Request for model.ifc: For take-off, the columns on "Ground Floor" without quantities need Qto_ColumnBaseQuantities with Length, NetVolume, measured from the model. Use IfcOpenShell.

First a look at what the model holds.

```python
import ifcopenshell
import ifcopenshell.util.element
import ifcopenshell.util.unit

model = ifcopenshell.open("model.ifc")
print(model.schema)
for unit_type in ("LENGTHUNIT", "AREAUNIT", "VOLUMEUNIT"):
    print(unit_type, ifcopenshell.util.unit.calculate_unit_scale(model, unit_type))
storey = next(s for s in model.by_type("IfcBuildingStorey") if s.Name == "Ground Floor")
columns = [e for e in ifcopenshell.util.element.get_decomposition(storey) if e.is_a("IfcColumn")]
for e in sorted(columns, key=lambda e: e.id()):
    print(e.id(), e.is_a(), e.Name, list(ifcopenshell.util.element.get_psets(e, qtos_only=True)), sep=" | ")
```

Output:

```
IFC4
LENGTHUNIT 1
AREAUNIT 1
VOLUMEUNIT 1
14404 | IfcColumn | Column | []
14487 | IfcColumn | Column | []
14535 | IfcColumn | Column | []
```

```python
import ifcopenshell
import ifcopenshell.api.pset
import ifcopenshell.geom
import ifcopenshell.util.element
import ifcopenshell.util.shape
import ifcopenshell.util.unit

model = ifcopenshell.open("model.ifc")
unit_scale = ifcopenshell.util.unit.calculate_unit_scale(model)
volume_scale = ifcopenshell.util.unit.calculate_unit_scale(model, "VOLUMEUNIT")
settings = ifcopenshell.geom.settings()

storey = next(s for s in model.by_type("IfcBuildingStorey") if s.Name == "Ground Floor")
columns = [e for e in ifcopenshell.util.element.get_decomposition(storey) if e.is_a("IfcColumn")]

for e in sorted(columns, key=lambda e: e.id()):
    if ifcopenshell.util.element.get_psets(e, qtos_only=True, should_inherit=False):
        continue
    # Geometry comes back in metres, in the element's own axes.
    shape = ifcopenshell.geom.create_shape(settings, e)
    values = {
        "Length": ifcopenshell.util.shape.get_z(shape.geometry) / unit_scale,
        "NetVolume": ifcopenshell.util.shape.get_volume(shape.geometry) / volume_scale,
    }
    qto = ifcopenshell.api.pset.add_qto(model, product=e, name="Qto_ColumnBaseQuantities")
    ifcopenshell.api.pset.edit_qto(model, qto=qto, properties=values)
    print(e.id(), {k: round(v, 3) for k, v in values.items()})

model.write("model-out.ifc")
```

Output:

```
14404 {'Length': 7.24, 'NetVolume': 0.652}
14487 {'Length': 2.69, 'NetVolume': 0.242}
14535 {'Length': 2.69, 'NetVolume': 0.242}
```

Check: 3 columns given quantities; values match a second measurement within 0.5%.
